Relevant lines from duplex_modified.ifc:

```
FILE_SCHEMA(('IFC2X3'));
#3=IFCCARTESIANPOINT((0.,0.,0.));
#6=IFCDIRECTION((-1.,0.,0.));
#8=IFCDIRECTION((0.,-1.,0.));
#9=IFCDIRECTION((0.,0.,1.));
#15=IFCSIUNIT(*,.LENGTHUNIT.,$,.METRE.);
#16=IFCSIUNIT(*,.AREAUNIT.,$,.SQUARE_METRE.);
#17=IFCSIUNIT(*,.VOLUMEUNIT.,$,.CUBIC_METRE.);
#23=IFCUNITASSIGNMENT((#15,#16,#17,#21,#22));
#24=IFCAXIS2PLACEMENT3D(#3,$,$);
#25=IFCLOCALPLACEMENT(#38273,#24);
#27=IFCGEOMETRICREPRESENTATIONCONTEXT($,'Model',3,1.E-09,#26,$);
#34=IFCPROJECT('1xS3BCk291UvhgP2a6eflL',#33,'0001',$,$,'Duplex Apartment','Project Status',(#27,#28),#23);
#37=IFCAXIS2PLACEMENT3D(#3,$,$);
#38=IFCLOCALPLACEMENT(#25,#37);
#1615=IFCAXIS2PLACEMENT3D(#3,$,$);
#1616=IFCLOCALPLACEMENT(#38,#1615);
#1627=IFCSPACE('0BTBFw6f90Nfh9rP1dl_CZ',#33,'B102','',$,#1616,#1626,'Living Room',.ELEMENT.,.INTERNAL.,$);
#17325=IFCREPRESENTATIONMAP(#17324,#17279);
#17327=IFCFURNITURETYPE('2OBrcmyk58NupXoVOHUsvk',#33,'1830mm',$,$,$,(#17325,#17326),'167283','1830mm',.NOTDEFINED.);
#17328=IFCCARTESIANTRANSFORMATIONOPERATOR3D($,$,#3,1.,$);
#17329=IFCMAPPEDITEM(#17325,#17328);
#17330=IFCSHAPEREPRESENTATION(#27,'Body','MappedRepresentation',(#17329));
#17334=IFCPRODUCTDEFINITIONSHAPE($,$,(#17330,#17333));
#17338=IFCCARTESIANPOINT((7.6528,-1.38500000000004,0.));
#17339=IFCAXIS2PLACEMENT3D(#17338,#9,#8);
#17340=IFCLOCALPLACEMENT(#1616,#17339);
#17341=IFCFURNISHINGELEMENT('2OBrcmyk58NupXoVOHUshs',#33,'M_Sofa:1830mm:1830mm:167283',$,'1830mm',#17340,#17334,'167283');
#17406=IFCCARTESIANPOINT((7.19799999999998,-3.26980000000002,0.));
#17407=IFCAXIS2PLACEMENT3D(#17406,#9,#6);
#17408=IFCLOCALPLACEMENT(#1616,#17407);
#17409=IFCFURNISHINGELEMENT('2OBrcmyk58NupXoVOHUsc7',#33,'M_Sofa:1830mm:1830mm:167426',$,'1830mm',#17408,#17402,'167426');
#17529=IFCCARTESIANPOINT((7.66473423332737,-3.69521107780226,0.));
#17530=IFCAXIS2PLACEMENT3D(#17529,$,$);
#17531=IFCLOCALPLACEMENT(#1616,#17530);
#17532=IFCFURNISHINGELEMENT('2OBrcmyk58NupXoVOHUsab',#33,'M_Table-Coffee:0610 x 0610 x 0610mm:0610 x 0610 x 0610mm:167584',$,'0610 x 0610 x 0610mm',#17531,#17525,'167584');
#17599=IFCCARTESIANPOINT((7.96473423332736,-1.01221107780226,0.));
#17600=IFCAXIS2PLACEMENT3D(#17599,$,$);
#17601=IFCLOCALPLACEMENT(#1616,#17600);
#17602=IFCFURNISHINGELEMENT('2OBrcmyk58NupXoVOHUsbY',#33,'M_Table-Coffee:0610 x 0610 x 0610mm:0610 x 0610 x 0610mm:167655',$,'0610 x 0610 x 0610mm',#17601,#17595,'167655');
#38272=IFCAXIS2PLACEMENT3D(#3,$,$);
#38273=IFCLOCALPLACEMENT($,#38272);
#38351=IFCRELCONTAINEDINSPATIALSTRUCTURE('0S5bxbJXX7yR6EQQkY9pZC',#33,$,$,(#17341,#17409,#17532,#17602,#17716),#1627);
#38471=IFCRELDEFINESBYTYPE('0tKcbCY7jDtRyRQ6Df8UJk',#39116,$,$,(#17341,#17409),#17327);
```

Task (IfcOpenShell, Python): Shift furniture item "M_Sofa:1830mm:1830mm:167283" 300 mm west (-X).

```python
import ifcopenshell
import ifcopenshell.api.geometry
import ifcopenshell.util.placement

model = ifcopenshell.open("duplex_modified.ifc")

item = model.by_guid("2OBrcmyk58NupXoVOHUshs")
matrix = ifcopenshell.util.placement.get_local_placement(item.ObjectPlacement)
matrix[0, 3] -= 0.3
ifcopenshell.api.geometry.edit_object_placement(model, product=item, matrix=matrix, is_si=False)

print(ifcopenshell.util.placement.get_local_placement(item.ObjectPlacement).round(3) + 0.0)

model.write("duplex_modified_v2.ifc")
```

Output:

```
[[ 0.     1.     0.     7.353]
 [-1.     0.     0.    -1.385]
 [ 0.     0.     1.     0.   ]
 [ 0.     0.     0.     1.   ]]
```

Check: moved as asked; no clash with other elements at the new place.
